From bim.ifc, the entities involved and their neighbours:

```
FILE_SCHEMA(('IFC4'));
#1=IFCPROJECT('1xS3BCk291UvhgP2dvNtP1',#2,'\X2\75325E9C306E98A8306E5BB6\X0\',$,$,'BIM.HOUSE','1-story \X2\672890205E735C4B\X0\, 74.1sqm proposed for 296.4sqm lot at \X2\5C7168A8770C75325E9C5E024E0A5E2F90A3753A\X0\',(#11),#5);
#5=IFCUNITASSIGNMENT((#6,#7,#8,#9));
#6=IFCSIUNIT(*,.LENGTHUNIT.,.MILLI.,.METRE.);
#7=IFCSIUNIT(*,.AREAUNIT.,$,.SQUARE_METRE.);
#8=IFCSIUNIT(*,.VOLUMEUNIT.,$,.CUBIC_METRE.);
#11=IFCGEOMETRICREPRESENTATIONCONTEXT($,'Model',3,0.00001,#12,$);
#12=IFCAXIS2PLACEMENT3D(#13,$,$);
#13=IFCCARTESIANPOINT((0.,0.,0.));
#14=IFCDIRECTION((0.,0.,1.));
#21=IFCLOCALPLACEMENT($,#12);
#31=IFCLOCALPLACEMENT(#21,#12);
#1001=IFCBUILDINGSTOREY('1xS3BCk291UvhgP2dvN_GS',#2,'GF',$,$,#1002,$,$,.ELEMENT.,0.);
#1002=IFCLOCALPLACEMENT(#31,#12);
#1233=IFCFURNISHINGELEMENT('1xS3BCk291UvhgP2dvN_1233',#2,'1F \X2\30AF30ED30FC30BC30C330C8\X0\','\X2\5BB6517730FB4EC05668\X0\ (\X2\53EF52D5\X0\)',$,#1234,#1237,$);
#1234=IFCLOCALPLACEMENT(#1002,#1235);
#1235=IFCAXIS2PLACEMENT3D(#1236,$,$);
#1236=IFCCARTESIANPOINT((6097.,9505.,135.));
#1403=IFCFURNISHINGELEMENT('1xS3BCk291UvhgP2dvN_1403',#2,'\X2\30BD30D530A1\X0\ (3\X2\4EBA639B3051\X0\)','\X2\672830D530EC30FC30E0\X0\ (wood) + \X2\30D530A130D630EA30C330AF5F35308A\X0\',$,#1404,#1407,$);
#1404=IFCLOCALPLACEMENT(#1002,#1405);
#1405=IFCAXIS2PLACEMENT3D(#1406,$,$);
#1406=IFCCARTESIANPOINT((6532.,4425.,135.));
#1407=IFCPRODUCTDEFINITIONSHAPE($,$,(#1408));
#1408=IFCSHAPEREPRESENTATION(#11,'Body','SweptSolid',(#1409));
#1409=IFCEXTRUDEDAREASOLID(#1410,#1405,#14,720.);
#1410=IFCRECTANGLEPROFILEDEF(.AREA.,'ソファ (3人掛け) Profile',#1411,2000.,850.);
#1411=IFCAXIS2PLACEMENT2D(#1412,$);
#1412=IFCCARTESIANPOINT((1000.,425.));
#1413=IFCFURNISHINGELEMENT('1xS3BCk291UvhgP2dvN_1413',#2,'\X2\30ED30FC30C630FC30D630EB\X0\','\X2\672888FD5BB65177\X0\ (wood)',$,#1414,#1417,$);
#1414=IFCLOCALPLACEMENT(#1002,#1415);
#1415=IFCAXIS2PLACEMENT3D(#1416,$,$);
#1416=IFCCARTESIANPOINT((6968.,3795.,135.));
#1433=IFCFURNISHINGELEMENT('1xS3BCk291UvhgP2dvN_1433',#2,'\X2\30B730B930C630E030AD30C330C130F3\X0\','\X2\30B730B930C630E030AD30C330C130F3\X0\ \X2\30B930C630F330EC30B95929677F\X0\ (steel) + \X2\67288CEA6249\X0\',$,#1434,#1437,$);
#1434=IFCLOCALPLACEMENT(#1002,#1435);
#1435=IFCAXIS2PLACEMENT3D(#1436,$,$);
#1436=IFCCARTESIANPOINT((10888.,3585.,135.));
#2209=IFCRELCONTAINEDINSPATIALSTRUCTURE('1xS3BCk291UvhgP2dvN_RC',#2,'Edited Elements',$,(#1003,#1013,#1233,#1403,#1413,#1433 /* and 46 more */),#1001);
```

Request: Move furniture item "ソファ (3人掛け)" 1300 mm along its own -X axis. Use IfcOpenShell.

```python
import ifcopenshell
import ifcopenshell.api.geometry
import ifcopenshell.util.placement
import ifcopenshell.util.unit

model = ifcopenshell.open("bim.ifc")
unit_scale = ifcopenshell.util.unit.calculate_unit_scale(model)

item = model.by_id(1403)
matrix = ifcopenshell.util.placement.get_local_placement(item.ObjectPlacement)
matrix[:3, 3] -= matrix[:3, 0] * 1.3 / unit_scale
ifcopenshell.api.geometry.edit_object_placement(model, product=item, matrix=matrix, is_si=False)

print(ifcopenshell.util.placement.get_local_placement(item.ObjectPlacement).round(3) + 0.0)

model.write("bim-out.ifc")
```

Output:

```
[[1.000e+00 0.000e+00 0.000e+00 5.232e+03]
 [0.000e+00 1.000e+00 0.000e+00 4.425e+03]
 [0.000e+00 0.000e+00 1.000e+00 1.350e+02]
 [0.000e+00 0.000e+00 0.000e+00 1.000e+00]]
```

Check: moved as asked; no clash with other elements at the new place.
